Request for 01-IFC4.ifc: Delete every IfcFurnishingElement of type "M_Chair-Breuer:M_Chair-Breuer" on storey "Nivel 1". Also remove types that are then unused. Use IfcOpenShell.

First a look at what the model holds.

```python
import ifcopenshell
import ifcopenshell.util.element

model = ifcopenshell.open("01-IFC4.ifc")
print(model.schema)
storey = next(s for s in model.by_type("IfcBuildingStorey") if s.Name == "Nivel 1")
furniture = [e for e in ifcopenshell.util.element.get_decomposition(storey) if e.is_a("IfcFurnishingElement")]
seen = {}
for e in furniture:
    element_type = ifcopenshell.util.element.get_type(e)
    name = element_type.Name if element_type not in (None, e) else None
    seen[name] = seen.get(name, 0) + 1
for name, count in sorted(seen.items(), key=str):
    print(count, "x", name)
```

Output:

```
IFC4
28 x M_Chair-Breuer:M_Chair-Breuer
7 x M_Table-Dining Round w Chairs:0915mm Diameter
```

```python
import ifcopenshell
import ifcopenshell.api.root
import ifcopenshell.util.element

model = ifcopenshell.open("01-IFC4.ifc")

storey = next(s for s in model.by_type("IfcBuildingStorey") if s.Name == "Nivel 1")
furniture = [e for e in ifcopenshell.util.element.get_decomposition(storey) if e.is_a("IfcFurnishingElement")]
targets = [e for e in furniture if (t := ifcopenshell.util.element.get_type(e)) not in (None, e) and t.Name == "M_Chair-Breuer:M_Chair-Breuer"]
types = {ifcopenshell.util.element.get_type(e) for e in targets} - {None, *targets}

for e in targets:
    ifcopenshell.api.root.remove_product(model, product=e)
print(len(targets), "removed")

unused = [t for t in types if not ifcopenshell.util.element.get_types(t)]
for t in unused:
    ifcopenshell.api.root.remove_product(model, product=t)
print(len(unused), "unused types removed")

model.write("01-IFC4_rev.ifc")
```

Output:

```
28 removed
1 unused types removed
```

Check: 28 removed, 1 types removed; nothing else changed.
